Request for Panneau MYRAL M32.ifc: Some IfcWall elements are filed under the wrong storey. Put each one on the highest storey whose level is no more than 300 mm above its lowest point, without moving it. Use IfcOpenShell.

First a look at what the model holds.

```python
import ifcopenshell
import ifcopenshell.util.element
import ifcopenshell.util.placement

model = ifcopenshell.open("Panneau MYRAL M32.ifc")
print(model.schema)
for storey in model.by_type("IfcBuildingStorey"):
    level = ifcopenshell.util.placement.get_storey_elevation(storey)
    count = sum(e.is_a("IfcWall") for e in ifcopenshell.util.element.get_contained(storey))
    print(storey.id(), storey.Name, round(level, 3), count, sep=" | ")
```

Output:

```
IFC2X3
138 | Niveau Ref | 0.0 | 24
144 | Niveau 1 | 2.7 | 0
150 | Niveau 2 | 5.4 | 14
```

```python
import ifcopenshell
import ifcopenshell.api.spatial
import ifcopenshell.geom
import ifcopenshell.util.element
import ifcopenshell.util.placement
import ifcopenshell.util.shape
import ifcopenshell.util.unit

model = ifcopenshell.open("Panneau MYRAL M32.ifc")
unit_scale = ifcopenshell.util.unit.calculate_unit_scale(model)
settings = ifcopenshell.geom.settings()

levels = sorted(
    ((ifcopenshell.util.placement.get_storey_elevation(s) * unit_scale, s) for s in model.by_type("IfcBuildingStorey")),
    key=lambda pair: pair[0],
)

for e in model.by_type("IfcWall"):
    current = e.ContainedInStructure[0].RelatingStructure if e.ContainedInStructure else None
    if current is None or not current.is_a("IfcBuildingStorey"):
        continue
    shape = ifcopenshell.geom.create_shape(settings, e)
    bottom = ifcopenshell.util.shape.get_shape_bottom_elevation(shape, shape.geometry)
    below = [s for level, s in levels if level <= bottom + 0.3]
    storey = below[-1] if below else levels[0][1]
    if storey != current:
        # assign_container keeps the world position.
        ifcopenshell.api.spatial.assign_container(model, products=[e], relating_structure=storey)
        print(e.id(), current.Name, "->", storey.Name)

model.write("Panneau MYRAL M32_edited.ifc")
```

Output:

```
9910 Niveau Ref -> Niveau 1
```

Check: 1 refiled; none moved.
